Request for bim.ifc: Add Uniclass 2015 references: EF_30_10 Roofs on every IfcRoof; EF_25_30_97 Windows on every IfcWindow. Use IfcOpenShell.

First a look at what the model holds.

```python
import ifcopenshell

model = ifcopenshell.open("bim.ifc")
print(model.schema)
print("classifications:", [c.Name for c in model.by_type("IfcClassification")])
for ifc_class in ("IfcDoor", "IfcRoof", "IfcStair", "IfcWall", "IfcWindow"):
    print(ifc_class, len(model.by_type(ifc_class)))
```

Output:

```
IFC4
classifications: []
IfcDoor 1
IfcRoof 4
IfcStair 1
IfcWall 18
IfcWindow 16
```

```python
import ifcopenshell
import ifcopenshell.api.classification

model = ifcopenshell.open("bim.ifc")

system = ifcopenshell.api.classification.add_classification(model, classification="Uniclass 2015")

codes = {
    "IfcRoof": ("EF_30_10", "Roofs"),
    "IfcWindow": ("EF_25_30_97", "Windows"),
}
for ifc_class, (code, name) in codes.items():
    products = model.by_type(ifc_class)
    ifcopenshell.api.classification.add_reference(
        model, products=products, classification=system, identification=code, name=name
    )
    print(code, len(products))

model.write("bim_updated.ifc")
```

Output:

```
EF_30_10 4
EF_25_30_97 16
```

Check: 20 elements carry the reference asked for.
